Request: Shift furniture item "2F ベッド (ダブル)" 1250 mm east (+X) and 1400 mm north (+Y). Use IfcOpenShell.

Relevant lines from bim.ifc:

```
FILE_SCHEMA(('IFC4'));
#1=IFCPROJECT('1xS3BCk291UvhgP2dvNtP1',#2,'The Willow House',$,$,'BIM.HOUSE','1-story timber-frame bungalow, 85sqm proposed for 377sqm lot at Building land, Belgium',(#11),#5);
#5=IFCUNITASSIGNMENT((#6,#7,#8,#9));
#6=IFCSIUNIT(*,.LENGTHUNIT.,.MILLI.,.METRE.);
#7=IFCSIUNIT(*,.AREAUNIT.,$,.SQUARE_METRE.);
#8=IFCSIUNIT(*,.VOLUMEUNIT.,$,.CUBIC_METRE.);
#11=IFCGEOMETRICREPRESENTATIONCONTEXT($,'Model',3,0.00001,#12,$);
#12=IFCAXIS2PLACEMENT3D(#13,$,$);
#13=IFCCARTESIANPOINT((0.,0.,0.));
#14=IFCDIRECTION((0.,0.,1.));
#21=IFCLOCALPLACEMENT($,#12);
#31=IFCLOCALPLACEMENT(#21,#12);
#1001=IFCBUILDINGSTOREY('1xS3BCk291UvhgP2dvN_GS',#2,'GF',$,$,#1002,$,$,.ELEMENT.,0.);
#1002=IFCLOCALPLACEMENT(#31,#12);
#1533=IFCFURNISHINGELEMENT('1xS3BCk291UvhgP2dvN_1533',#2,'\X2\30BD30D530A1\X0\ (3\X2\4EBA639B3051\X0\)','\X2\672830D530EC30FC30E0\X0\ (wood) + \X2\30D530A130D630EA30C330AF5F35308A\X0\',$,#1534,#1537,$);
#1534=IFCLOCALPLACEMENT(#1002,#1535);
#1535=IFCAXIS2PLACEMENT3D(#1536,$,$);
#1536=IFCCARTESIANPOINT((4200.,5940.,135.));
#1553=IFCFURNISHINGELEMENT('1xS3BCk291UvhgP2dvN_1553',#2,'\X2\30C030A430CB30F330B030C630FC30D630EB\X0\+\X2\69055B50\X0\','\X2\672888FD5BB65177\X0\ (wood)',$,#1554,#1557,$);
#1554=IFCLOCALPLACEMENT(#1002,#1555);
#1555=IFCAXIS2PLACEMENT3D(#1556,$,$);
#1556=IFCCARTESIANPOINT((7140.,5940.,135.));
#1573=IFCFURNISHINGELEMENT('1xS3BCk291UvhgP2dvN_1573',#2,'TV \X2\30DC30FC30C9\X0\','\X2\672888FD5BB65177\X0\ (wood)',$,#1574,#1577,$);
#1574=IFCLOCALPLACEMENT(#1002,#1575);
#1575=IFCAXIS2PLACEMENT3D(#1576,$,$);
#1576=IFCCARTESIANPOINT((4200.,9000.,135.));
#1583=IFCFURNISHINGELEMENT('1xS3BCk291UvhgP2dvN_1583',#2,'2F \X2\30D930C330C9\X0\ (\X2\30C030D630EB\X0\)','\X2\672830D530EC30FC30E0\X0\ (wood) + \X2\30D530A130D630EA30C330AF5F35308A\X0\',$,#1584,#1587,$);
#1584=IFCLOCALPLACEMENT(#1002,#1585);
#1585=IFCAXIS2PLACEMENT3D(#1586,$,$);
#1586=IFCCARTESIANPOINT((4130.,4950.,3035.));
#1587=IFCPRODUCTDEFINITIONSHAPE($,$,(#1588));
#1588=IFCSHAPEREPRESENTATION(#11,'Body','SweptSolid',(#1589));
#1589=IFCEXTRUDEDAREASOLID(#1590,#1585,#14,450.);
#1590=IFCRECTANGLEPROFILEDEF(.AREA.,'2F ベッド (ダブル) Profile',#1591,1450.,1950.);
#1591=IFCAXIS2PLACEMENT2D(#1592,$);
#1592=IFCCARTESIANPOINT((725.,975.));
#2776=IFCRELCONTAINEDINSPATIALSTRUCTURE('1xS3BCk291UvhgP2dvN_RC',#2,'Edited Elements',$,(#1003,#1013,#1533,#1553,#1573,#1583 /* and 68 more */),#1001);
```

```python
import ifcopenshell
import ifcopenshell.api.geometry
import ifcopenshell.util.placement
import ifcopenshell.util.unit

model = ifcopenshell.open("bim.ifc")
unit_scale = ifcopenshell.util.unit.calculate_unit_scale(model)

item = model.by_id(1583)
matrix = ifcopenshell.util.placement.get_local_placement(item.ObjectPlacement)
matrix[0, 3] += 1.25 / unit_scale
matrix[1, 3] += 1.4 / unit_scale
ifcopenshell.api.geometry.edit_object_placement(model, product=item, matrix=matrix, is_si=False)

print(ifcopenshell.util.placement.get_local_placement(item.ObjectPlacement).round(3) + 0.0)

model.write("bim_v2.ifc")
```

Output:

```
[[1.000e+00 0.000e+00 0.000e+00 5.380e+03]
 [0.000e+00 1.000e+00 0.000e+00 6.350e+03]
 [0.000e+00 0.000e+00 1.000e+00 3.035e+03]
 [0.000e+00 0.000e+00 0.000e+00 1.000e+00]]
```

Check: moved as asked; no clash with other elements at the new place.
